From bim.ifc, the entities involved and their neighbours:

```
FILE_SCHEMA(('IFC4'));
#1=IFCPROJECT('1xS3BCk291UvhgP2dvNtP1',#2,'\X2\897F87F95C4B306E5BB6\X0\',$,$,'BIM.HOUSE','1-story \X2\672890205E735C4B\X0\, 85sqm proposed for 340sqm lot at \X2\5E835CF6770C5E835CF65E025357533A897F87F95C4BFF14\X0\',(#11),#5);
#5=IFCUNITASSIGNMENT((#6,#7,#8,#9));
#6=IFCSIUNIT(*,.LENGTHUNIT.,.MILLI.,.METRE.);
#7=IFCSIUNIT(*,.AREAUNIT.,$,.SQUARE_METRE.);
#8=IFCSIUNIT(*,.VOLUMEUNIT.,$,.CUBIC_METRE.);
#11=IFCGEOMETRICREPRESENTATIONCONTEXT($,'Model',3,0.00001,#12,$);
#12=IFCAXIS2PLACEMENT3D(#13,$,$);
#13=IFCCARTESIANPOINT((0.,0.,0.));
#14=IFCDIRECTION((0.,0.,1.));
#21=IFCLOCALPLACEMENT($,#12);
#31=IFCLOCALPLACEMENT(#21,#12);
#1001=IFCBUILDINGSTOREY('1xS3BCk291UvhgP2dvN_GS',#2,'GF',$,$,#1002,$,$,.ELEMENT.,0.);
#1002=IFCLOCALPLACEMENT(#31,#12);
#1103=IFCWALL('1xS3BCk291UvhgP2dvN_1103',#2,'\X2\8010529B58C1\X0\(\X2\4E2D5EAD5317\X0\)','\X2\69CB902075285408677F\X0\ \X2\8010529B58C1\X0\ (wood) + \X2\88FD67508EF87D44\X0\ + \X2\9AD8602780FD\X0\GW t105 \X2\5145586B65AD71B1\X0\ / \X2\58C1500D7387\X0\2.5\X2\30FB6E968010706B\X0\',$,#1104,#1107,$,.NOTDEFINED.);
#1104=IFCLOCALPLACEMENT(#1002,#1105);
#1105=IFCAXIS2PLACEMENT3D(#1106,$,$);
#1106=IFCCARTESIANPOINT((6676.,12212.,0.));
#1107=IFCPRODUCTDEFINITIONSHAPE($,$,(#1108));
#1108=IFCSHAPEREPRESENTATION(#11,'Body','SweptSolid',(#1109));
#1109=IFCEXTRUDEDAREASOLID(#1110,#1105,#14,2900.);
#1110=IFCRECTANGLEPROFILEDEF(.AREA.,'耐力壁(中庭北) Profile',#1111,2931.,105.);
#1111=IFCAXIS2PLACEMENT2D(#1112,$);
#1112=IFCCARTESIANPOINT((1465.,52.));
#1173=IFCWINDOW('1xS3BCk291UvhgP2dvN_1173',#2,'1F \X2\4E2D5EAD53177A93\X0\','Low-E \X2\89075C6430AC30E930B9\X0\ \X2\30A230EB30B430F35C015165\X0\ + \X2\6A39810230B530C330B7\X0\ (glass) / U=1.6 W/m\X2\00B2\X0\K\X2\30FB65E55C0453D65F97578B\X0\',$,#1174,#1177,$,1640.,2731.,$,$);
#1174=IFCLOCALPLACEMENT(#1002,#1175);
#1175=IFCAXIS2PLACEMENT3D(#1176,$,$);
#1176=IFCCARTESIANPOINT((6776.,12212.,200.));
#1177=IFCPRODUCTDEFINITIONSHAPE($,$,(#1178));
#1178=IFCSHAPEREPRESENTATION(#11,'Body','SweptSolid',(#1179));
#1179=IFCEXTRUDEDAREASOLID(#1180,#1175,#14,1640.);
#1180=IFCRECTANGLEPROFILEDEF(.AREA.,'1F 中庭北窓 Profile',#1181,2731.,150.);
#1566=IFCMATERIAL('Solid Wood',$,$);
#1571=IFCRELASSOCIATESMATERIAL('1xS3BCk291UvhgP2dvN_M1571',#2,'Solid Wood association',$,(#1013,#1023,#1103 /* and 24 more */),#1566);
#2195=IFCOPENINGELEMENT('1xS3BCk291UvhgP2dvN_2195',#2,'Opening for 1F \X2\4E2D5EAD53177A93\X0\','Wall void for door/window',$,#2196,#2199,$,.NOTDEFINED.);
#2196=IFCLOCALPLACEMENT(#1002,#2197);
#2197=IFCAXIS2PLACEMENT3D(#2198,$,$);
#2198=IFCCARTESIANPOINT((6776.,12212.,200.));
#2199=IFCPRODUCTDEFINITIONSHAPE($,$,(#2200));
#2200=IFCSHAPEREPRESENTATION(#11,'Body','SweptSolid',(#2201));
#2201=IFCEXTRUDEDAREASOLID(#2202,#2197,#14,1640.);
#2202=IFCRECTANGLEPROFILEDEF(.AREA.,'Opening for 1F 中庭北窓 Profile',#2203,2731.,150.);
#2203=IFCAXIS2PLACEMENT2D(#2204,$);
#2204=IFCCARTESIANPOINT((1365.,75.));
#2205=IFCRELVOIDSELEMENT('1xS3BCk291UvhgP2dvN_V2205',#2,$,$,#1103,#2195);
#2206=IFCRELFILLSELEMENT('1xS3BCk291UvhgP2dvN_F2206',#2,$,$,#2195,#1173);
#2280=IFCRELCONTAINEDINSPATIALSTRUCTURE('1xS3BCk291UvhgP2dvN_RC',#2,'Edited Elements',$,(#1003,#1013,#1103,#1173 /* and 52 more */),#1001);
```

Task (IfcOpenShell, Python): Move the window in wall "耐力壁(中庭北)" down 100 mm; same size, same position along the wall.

```python
import numpy as np
import ifcopenshell
import ifcopenshell.api.geometry
import ifcopenshell.util.placement
import ifcopenshell.util.unit

model = ifcopenshell.open("bim.ifc")
unit_scale = ifcopenshell.util.unit.calculate_unit_scale(model)

window = model.by_id(1173)
opening = window.FillsVoids[0].RelatingOpeningElement
dz = -0.1 / unit_scale

shift = np.array([0.0, 0.0, dz])
# The window is not placed relative to its opening, so move both.
for product in (opening, window):
    matrix = ifcopenshell.util.placement.get_local_placement(product.ObjectPlacement)
    matrix[:3, 3] += shift
    ifcopenshell.api.geometry.edit_object_placement(model, product=product, matrix=matrix, is_si=False)

print(f"moved by {dz * unit_scale:+.3f} m")

model.write("bim_updated.ifc")
```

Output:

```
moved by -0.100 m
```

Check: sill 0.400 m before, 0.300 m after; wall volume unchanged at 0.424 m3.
